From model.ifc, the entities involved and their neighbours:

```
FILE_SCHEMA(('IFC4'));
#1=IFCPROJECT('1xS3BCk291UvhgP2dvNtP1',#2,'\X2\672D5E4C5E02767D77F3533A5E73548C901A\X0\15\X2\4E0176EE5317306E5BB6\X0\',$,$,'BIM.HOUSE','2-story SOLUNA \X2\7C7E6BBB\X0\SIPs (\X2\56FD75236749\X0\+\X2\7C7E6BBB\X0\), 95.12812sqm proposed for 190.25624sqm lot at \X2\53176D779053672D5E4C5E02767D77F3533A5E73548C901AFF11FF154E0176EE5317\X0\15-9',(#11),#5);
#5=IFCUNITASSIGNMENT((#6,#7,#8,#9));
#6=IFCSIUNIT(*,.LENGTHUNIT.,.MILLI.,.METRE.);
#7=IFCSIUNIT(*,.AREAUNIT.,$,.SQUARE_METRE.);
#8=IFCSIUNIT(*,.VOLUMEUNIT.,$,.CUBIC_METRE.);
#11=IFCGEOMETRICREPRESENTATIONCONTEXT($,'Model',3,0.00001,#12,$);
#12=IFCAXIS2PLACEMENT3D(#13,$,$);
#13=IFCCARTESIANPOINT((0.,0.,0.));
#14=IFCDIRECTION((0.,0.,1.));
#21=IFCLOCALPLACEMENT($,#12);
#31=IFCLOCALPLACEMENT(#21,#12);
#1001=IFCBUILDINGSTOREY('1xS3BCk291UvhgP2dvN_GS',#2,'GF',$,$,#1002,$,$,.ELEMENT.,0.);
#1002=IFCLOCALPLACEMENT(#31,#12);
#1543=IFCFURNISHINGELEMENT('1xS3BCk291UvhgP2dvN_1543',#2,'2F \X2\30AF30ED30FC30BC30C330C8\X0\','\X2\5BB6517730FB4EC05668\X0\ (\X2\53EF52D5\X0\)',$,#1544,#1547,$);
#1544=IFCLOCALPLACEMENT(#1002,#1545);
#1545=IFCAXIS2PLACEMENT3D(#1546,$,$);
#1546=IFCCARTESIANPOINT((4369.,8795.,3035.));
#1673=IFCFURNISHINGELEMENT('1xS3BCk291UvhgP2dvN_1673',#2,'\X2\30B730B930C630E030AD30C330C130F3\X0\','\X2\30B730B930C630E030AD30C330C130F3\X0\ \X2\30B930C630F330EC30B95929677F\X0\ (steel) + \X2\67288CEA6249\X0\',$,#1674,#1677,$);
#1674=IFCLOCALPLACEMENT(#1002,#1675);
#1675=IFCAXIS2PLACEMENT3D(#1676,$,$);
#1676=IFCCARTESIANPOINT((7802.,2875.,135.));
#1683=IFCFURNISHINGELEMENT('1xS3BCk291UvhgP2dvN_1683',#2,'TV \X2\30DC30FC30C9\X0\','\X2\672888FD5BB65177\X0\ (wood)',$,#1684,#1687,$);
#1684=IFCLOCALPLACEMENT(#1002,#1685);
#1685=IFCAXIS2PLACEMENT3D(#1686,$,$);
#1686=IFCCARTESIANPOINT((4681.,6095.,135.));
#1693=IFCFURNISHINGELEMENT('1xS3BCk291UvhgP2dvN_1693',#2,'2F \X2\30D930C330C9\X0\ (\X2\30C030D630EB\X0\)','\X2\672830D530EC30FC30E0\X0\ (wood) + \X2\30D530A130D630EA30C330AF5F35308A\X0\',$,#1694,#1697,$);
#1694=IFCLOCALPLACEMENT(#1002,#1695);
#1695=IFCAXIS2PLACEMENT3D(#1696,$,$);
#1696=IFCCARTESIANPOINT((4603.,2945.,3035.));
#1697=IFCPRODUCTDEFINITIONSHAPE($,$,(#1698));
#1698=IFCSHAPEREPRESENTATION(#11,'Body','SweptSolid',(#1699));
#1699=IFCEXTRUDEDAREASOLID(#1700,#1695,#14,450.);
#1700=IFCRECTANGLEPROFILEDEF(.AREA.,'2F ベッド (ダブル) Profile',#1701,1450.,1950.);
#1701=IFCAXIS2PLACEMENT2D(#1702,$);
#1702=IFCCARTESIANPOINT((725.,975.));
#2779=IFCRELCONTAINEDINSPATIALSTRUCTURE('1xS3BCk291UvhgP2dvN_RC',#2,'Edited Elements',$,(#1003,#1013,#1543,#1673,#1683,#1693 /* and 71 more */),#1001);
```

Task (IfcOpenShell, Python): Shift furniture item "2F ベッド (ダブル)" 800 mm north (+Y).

```python
import ifcopenshell
import ifcopenshell.api.geometry
import ifcopenshell.util.placement
import ifcopenshell.util.unit

model = ifcopenshell.open("model.ifc")
unit_scale = ifcopenshell.util.unit.calculate_unit_scale(model)

item = model.by_guid("1xS3BCk291UvhgP2dvN_1693")
matrix = ifcopenshell.util.placement.get_local_placement(item.ObjectPlacement)
matrix[1, 3] += 0.8 / unit_scale
ifcopenshell.api.geometry.edit_object_placement(model, product=item, matrix=matrix, is_si=False)

print(ifcopenshell.util.placement.get_local_placement(item.ObjectPlacement).round(3) + 0.0)

model.write("model-out.ifc")
```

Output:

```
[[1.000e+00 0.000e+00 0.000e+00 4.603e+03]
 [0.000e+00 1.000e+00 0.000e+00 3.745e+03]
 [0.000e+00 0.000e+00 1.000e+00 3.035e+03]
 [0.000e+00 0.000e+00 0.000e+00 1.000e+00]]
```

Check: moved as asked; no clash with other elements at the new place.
